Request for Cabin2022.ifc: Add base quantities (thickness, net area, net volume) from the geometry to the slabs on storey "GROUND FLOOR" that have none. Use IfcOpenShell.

First a look at what the model holds.

```python
import ifcopenshell
import ifcopenshell.util.element
import ifcopenshell.util.unit

model = ifcopenshell.open("Cabin2022.ifc")
print(model.schema)
for unit_type in ("LENGTHUNIT", "AREAUNIT", "VOLUMEUNIT"):
    print(unit_type, ifcopenshell.util.unit.calculate_unit_scale(model, unit_type))
storey = next(s for s in model.by_type("IfcBuildingStorey") if s.Name == "GROUND FLOOR")
slabs = [e for e in ifcopenshell.util.element.get_decomposition(storey) if e.is_a("IfcSlab")]
for e in sorted(slabs, key=lambda e: e.id()):
    print(e.id(), e.is_a(), e.Name, list(ifcopenshell.util.element.get_psets(e, qtos_only=True)), sep=" | ")
```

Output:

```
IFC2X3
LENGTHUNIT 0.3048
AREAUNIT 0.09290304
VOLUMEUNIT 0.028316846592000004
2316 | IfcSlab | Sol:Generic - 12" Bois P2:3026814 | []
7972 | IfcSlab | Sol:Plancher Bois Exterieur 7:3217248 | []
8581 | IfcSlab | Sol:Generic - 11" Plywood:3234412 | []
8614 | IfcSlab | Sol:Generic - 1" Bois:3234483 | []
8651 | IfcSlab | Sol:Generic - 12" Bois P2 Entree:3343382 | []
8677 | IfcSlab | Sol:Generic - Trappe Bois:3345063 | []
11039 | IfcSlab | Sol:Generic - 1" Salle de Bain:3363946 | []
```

```python
import ifcopenshell
import ifcopenshell.api.pset
import ifcopenshell.geom
import ifcopenshell.util.element
import ifcopenshell.util.shape
import ifcopenshell.util.unit

model = ifcopenshell.open("Cabin2022.ifc")
unit_scale = ifcopenshell.util.unit.calculate_unit_scale(model)
area_scale = ifcopenshell.util.unit.calculate_unit_scale(model, "AREAUNIT")
volume_scale = ifcopenshell.util.unit.calculate_unit_scale(model, "VOLUMEUNIT")
settings = ifcopenshell.geom.settings()

storey = next(s for s in model.by_type("IfcBuildingStorey") if s.Name == "GROUND FLOOR")
slabs = [e for e in ifcopenshell.util.element.get_decomposition(storey) if e.is_a("IfcSlab")]

for e in sorted(slabs, key=lambda e: e.id()):
    if ifcopenshell.util.element.get_psets(e, qtos_only=True, should_inherit=False):
        continue
    # Geometry comes back in metres, in the element's own axes.
    shape = ifcopenshell.geom.create_shape(settings, e)
    values = {
        "Width": ifcopenshell.util.shape.get_z(shape.geometry) / unit_scale,
        "NetArea": ifcopenshell.util.shape.get_footprint_area(shape.geometry) / area_scale,
        "NetVolume": ifcopenshell.util.shape.get_volume(shape.geometry) / volume_scale,
    }
    qto = ifcopenshell.api.pset.add_qto(model, product=e, name="BaseQuantities")
    ifcopenshell.api.pset.edit_qto(model, qto=qto, properties=values)
    print(e.id(), {k: round(v, 3) for k, v in values.items()})

model.write("Cabin2022_edited.ifc")
```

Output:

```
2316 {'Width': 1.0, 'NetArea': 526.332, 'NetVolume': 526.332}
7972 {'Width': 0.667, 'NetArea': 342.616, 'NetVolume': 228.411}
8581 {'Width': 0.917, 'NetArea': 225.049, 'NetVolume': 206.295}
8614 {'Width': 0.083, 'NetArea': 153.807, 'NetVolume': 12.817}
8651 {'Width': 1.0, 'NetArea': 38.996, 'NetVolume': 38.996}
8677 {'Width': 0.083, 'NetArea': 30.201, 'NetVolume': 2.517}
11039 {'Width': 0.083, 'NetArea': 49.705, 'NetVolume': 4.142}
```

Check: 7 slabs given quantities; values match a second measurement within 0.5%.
